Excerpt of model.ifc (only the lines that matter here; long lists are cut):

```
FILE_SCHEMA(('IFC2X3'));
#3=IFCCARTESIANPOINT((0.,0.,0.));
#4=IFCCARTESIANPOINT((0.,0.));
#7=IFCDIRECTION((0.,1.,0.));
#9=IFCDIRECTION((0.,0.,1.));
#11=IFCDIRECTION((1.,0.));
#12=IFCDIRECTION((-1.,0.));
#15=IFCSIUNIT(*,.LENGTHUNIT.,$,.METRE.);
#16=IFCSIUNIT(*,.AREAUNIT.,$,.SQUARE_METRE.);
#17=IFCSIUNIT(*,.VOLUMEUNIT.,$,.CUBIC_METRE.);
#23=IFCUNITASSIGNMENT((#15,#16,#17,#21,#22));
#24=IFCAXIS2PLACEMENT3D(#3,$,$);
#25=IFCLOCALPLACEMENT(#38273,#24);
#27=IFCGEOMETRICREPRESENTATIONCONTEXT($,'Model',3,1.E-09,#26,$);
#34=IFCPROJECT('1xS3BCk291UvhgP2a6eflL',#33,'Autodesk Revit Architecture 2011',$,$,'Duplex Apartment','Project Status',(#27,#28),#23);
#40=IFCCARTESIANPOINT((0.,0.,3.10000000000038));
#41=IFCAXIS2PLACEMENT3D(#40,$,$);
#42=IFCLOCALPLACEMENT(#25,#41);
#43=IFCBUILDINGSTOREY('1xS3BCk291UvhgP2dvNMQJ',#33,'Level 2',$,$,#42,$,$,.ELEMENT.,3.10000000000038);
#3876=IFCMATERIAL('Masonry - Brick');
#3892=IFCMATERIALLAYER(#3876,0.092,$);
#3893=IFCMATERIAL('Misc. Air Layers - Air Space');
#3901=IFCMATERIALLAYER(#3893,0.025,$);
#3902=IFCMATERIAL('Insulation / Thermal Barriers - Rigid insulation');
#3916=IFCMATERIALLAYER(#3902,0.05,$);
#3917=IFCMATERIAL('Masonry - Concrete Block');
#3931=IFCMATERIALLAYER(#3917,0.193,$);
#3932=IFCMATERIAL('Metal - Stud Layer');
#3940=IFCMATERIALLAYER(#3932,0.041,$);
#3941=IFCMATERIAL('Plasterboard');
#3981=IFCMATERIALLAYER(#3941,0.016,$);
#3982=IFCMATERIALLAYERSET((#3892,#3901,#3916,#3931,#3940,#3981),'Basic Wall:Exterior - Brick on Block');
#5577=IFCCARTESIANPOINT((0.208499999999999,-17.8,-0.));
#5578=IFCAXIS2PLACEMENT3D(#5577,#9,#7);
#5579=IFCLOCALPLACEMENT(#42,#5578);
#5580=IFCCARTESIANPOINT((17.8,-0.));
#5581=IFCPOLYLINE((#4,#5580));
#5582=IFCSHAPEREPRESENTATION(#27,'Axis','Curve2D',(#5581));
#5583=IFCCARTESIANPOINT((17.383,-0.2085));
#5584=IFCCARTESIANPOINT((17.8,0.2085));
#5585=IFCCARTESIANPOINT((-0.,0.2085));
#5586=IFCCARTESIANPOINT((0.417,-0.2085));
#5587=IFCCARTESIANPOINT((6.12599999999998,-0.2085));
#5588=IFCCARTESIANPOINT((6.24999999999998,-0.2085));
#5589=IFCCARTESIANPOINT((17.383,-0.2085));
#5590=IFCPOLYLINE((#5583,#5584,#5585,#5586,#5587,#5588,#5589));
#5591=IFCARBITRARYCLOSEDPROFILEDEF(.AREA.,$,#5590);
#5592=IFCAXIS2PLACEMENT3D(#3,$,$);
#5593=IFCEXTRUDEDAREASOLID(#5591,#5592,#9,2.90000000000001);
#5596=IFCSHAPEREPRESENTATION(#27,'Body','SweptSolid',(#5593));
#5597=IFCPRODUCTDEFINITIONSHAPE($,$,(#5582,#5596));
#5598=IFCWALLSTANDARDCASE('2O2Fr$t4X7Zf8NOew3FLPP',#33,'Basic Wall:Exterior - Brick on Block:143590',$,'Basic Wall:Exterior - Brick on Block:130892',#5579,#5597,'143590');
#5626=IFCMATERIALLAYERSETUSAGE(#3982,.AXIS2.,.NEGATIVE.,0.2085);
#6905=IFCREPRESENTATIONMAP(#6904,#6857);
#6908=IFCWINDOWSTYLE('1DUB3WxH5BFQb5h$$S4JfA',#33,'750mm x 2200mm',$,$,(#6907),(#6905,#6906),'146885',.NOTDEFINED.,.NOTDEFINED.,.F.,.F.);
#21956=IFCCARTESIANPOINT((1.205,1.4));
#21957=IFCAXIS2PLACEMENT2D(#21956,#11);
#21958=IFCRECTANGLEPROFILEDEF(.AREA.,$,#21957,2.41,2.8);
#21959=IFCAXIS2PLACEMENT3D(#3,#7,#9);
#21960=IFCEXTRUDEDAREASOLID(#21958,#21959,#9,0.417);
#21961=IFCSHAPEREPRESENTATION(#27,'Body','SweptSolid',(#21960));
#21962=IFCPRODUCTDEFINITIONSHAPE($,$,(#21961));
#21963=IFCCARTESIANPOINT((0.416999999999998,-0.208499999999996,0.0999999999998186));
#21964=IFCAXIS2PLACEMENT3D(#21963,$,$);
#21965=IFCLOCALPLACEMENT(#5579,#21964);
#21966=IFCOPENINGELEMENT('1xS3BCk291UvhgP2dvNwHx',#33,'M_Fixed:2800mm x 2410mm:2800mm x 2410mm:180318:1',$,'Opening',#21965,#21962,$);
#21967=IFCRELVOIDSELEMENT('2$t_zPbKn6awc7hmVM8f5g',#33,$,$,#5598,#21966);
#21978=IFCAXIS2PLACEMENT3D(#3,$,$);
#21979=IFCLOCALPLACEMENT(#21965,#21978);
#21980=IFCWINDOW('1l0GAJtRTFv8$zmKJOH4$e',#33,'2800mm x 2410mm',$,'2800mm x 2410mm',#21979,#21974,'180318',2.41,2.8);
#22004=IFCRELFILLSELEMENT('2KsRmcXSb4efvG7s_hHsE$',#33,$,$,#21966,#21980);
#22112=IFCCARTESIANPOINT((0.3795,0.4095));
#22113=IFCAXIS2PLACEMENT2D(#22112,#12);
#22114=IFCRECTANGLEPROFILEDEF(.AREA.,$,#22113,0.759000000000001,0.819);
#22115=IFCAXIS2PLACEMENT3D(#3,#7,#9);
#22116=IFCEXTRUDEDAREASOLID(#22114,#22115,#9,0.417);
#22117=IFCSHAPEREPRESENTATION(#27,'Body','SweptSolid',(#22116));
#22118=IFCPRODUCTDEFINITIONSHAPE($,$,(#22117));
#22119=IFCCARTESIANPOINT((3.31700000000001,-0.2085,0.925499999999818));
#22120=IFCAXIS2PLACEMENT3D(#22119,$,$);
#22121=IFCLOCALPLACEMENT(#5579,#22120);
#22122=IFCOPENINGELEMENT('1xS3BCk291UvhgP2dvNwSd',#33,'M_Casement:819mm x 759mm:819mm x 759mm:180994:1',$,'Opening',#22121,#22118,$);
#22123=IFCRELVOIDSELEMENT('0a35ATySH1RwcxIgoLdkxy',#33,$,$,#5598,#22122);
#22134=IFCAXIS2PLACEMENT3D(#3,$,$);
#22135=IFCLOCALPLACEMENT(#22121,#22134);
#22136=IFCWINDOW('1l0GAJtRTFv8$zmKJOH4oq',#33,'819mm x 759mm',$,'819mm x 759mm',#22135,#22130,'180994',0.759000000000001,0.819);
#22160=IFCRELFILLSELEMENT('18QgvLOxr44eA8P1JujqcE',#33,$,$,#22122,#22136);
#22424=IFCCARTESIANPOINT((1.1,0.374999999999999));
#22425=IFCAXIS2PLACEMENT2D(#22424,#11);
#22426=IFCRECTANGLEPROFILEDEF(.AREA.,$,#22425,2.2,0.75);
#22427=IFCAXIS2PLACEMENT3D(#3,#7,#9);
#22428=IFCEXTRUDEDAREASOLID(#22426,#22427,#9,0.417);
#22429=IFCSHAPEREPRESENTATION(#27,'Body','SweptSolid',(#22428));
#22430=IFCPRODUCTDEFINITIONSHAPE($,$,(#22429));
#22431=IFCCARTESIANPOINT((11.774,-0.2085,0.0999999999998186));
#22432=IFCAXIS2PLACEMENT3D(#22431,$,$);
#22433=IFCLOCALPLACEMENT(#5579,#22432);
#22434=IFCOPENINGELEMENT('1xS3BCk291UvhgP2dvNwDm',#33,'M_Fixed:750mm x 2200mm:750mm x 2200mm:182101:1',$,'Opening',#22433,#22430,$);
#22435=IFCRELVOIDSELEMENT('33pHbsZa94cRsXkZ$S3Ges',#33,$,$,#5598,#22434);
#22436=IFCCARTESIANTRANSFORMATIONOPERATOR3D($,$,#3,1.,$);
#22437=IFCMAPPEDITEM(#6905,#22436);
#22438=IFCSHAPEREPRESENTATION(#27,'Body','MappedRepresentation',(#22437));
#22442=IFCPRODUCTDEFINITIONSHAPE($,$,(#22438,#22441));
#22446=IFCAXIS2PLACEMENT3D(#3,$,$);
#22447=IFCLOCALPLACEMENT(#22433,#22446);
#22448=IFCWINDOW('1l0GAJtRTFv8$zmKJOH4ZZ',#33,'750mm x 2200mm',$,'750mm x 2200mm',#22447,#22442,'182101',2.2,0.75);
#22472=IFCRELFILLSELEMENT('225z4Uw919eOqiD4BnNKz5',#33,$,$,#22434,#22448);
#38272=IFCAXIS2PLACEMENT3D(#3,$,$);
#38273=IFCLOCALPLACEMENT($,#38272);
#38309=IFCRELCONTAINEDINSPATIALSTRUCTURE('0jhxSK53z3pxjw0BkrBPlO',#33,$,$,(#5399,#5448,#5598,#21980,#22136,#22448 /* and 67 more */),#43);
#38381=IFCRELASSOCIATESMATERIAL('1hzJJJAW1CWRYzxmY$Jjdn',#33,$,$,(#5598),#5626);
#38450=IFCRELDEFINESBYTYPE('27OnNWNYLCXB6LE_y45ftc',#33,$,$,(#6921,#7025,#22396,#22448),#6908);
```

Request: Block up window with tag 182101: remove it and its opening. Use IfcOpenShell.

```python
import ifcopenshell
import ifcopenshell.api.feature
import ifcopenshell.api.root
import ifcopenshell.geom
import ifcopenshell.util.shape

model = ifcopenshell.open("model.ifc")
settings = ifcopenshell.geom.settings()


def volume(element):
    """Net volume in cubic metres, openings subtracted."""
    shape = ifcopenshell.geom.create_shape(settings, element)
    return ifcopenshell.util.shape.get_volume(shape.geometry)


window = model.by_id(22448)
opening = window.FillsVoids[0].RelatingOpeningElement
wall = opening.VoidsElements[0].RelatingBuildingElement
before = volume(wall)

ifcopenshell.api.root.remove_product(model, product=window)
ifcopenshell.api.feature.remove_feature(model, feature=opening)

after = volume(wall)

print(f"wall volume {before:.3f} -> {after:.3f} m3")

model.write("model_v2.ifc")
```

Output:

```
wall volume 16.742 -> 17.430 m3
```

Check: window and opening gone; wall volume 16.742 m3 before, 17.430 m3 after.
